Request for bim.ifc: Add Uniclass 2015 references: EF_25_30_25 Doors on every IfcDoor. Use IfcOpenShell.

First a look at what the model holds.

```python
import ifcopenshell

model = ifcopenshell.open("bim.ifc")
print(model.schema)
print("classifications:", [c.Name for c in model.by_type("IfcClassification")])
for ifc_class in ("IfcDoor", "IfcRoof", "IfcStair", "IfcWall", "IfcWindow"):
    print(ifc_class, len(model.by_type(ifc_class)))
```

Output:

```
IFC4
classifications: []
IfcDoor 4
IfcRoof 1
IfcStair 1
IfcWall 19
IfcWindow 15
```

```python
import ifcopenshell
import ifcopenshell.api.classification

model = ifcopenshell.open("bim.ifc")

system = ifcopenshell.api.classification.add_classification(model, classification="Uniclass 2015")

codes = {
    "IfcDoor": ("EF_25_30_25", "Doors"),
}
for ifc_class, (code, name) in codes.items():
    products = model.by_type(ifc_class)
    ifcopenshell.api.classification.add_reference(
        model, products=products, classification=system, identification=code, name=name
    )
    print(code, len(products))

model.write("bim_edited.ifc")
```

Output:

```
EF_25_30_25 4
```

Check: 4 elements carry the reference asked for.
